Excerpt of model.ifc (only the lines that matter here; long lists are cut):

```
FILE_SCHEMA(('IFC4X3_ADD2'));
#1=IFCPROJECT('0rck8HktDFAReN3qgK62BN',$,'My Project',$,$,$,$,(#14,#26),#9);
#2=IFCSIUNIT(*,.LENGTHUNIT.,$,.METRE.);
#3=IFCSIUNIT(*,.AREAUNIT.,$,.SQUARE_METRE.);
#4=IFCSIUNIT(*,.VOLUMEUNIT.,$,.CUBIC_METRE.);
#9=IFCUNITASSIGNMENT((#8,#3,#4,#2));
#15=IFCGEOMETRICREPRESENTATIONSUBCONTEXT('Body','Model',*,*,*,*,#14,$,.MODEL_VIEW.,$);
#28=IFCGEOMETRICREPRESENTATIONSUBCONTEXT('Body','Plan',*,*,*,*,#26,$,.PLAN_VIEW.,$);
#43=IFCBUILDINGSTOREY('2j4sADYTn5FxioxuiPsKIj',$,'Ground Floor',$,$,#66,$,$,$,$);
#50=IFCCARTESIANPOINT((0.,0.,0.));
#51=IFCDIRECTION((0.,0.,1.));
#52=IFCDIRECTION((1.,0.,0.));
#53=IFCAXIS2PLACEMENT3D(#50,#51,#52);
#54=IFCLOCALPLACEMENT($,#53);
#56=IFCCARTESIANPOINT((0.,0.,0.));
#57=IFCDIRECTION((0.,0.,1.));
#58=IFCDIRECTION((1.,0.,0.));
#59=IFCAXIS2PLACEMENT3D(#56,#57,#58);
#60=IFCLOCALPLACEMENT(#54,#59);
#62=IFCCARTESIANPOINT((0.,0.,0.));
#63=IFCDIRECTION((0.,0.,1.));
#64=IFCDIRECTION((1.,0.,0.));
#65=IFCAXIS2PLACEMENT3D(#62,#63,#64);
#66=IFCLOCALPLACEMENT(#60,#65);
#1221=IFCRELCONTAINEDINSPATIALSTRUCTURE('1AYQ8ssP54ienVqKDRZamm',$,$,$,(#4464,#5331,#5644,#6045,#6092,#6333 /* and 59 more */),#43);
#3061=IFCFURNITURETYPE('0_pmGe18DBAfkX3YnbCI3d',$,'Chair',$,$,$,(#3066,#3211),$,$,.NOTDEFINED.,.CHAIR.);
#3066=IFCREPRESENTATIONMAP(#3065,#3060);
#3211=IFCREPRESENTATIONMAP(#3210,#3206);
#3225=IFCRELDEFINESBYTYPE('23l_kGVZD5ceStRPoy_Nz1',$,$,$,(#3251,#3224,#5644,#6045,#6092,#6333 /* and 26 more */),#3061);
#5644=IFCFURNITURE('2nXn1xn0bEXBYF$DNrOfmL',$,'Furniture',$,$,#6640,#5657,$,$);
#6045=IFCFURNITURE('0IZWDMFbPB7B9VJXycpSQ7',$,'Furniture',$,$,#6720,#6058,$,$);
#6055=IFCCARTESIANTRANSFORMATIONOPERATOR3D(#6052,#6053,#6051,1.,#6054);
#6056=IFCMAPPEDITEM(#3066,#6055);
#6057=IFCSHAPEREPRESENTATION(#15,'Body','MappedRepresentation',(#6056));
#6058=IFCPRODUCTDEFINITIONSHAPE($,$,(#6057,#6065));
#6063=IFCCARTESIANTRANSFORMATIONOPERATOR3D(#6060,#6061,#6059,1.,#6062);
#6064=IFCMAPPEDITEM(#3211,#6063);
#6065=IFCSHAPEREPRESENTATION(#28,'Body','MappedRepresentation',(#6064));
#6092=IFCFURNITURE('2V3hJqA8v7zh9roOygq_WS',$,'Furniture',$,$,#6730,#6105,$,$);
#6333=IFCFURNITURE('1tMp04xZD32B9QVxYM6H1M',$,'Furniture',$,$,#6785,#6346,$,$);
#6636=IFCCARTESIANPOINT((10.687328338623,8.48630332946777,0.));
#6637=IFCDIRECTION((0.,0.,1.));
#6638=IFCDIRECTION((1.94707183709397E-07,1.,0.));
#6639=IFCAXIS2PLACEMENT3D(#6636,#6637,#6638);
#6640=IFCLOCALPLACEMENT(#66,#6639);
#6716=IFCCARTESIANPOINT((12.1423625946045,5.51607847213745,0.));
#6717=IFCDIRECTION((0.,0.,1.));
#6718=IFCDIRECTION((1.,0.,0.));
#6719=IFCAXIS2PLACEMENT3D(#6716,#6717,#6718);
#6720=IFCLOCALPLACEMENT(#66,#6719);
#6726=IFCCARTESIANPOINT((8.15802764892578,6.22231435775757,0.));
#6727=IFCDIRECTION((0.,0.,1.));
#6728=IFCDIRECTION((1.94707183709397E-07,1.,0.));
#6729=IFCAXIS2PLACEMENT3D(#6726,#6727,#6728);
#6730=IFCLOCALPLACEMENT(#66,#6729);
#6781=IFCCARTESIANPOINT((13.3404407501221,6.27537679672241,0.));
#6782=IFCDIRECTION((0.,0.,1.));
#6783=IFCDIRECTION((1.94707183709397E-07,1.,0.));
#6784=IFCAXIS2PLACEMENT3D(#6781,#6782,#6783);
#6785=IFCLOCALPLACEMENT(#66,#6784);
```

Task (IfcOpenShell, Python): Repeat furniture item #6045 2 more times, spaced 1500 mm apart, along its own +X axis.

```python
import ifcopenshell
import ifcopenshell.api.geometry
import ifcopenshell.api.root
import ifcopenshell.util.element
import ifcopenshell.util.placement
import ifcopenshell.util.unit

model = ifcopenshell.open("model.ifc")
unit_scale = ifcopenshell.util.unit.calculate_unit_scale(model)

source = model.by_guid("0IZWDMFbPB7B9VJXycpSQ7")
base = ifcopenshell.util.placement.get_local_placement(source.ObjectPlacement)
step = base[:3, 0] * 1.5 / unit_scale

for i in range(1, 3):
    copy = ifcopenshell.api.root.copy_class(model, product=source)
    copy.Representation = ifcopenshell.util.element.copy_deep(
        model, source.Representation, exclude=["IfcGeometricRepresentationContext", "IfcRepresentationMap"]
    )
    matrix = base.copy()
    matrix[:3, 3] += i * step
    print("added at", matrix[:3, 3].round(3) + 0.0)
    ifcopenshell.api.geometry.edit_object_placement(model, product=copy, matrix=matrix, is_si=False)

model.write("model_rev.ifc")
```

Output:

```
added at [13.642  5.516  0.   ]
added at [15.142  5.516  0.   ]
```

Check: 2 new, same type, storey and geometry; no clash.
